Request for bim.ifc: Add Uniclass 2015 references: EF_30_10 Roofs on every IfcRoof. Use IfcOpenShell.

First a look at what the model holds.

```python
import ifcopenshell

model = ifcopenshell.open("bim.ifc")
print(model.schema)
print("classifications:", [c.Name for c in model.by_type("IfcClassification")])
for ifc_class in ("IfcDoor", "IfcRoof", "IfcStair", "IfcWall", "IfcWindow"):
    print(ifc_class, len(model.by_type(ifc_class)))
```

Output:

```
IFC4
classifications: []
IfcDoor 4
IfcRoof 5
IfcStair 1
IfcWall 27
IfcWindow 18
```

```python
import ifcopenshell
import ifcopenshell.api.classification

model = ifcopenshell.open("bim.ifc")

system = ifcopenshell.api.classification.add_classification(model, classification="Uniclass 2015")

codes = {
    "IfcRoof": ("EF_30_10", "Roofs"),
}
for ifc_class, (code, name) in codes.items():
    products = model.by_type(ifc_class)
    ifcopenshell.api.classification.add_reference(
        model, products=products, classification=system, identification=code, name=name
    )
    print(code, len(products))

model.write("bim_updated.ifc")
```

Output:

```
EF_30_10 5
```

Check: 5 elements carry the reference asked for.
